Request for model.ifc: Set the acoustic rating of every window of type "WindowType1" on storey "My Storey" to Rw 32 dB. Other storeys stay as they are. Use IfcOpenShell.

First a look at what the model holds.

```python
import ifcopenshell
import ifcopenshell.util.element

model = ifcopenshell.open("model.ifc")
print(model.schema)
storey = next(s for s in model.by_type("IfcBuildingStorey") if s.Name == "My Storey")
windows = [e for e in ifcopenshell.util.element.get_decomposition(storey) if e.is_a("IfcWindow")]
seen = {}
for e in windows:
    element_type = ifcopenshell.util.element.get_type(e)
    key = (element_type.Name if element_type != e and element_type else None, ifcopenshell.util.element.get_pset(e, "Pset_WindowCommon", "AcousticRating"))
    seen[key] = seen.get(key, 0) + 1
for (name, value), count in sorted(seen.items(), key=str):
    print(count, "x", name, "|", value)
```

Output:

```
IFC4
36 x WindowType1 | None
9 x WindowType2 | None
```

```python
import ifcopenshell
import ifcopenshell.api.pset
import ifcopenshell.util.element

model = ifcopenshell.open("model.ifc")

storey = next(s for s in model.by_type("IfcBuildingStorey") if s.Name == "My Storey")
windows = [e for e in ifcopenshell.util.element.get_decomposition(storey) if e.is_a("IfcWindow")]

count = 0
for e in windows:
    element_type = ifcopenshell.util.element.get_type(e)
    if element_type in (None, e) or element_type.Name != "WindowType1":
        continue
    # add_pset returns the element's existing set when there is one.
    pset = ifcopenshell.api.pset.add_pset(model, product=e, name="Pset_WindowCommon")
    ifcopenshell.api.pset.edit_pset(model, pset=pset, properties={"AcousticRating": "Rw 32 dB"})
    count += 1

print(count, "windows updated")

model.write("model_v2.ifc")
```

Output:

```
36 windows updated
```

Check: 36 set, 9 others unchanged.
